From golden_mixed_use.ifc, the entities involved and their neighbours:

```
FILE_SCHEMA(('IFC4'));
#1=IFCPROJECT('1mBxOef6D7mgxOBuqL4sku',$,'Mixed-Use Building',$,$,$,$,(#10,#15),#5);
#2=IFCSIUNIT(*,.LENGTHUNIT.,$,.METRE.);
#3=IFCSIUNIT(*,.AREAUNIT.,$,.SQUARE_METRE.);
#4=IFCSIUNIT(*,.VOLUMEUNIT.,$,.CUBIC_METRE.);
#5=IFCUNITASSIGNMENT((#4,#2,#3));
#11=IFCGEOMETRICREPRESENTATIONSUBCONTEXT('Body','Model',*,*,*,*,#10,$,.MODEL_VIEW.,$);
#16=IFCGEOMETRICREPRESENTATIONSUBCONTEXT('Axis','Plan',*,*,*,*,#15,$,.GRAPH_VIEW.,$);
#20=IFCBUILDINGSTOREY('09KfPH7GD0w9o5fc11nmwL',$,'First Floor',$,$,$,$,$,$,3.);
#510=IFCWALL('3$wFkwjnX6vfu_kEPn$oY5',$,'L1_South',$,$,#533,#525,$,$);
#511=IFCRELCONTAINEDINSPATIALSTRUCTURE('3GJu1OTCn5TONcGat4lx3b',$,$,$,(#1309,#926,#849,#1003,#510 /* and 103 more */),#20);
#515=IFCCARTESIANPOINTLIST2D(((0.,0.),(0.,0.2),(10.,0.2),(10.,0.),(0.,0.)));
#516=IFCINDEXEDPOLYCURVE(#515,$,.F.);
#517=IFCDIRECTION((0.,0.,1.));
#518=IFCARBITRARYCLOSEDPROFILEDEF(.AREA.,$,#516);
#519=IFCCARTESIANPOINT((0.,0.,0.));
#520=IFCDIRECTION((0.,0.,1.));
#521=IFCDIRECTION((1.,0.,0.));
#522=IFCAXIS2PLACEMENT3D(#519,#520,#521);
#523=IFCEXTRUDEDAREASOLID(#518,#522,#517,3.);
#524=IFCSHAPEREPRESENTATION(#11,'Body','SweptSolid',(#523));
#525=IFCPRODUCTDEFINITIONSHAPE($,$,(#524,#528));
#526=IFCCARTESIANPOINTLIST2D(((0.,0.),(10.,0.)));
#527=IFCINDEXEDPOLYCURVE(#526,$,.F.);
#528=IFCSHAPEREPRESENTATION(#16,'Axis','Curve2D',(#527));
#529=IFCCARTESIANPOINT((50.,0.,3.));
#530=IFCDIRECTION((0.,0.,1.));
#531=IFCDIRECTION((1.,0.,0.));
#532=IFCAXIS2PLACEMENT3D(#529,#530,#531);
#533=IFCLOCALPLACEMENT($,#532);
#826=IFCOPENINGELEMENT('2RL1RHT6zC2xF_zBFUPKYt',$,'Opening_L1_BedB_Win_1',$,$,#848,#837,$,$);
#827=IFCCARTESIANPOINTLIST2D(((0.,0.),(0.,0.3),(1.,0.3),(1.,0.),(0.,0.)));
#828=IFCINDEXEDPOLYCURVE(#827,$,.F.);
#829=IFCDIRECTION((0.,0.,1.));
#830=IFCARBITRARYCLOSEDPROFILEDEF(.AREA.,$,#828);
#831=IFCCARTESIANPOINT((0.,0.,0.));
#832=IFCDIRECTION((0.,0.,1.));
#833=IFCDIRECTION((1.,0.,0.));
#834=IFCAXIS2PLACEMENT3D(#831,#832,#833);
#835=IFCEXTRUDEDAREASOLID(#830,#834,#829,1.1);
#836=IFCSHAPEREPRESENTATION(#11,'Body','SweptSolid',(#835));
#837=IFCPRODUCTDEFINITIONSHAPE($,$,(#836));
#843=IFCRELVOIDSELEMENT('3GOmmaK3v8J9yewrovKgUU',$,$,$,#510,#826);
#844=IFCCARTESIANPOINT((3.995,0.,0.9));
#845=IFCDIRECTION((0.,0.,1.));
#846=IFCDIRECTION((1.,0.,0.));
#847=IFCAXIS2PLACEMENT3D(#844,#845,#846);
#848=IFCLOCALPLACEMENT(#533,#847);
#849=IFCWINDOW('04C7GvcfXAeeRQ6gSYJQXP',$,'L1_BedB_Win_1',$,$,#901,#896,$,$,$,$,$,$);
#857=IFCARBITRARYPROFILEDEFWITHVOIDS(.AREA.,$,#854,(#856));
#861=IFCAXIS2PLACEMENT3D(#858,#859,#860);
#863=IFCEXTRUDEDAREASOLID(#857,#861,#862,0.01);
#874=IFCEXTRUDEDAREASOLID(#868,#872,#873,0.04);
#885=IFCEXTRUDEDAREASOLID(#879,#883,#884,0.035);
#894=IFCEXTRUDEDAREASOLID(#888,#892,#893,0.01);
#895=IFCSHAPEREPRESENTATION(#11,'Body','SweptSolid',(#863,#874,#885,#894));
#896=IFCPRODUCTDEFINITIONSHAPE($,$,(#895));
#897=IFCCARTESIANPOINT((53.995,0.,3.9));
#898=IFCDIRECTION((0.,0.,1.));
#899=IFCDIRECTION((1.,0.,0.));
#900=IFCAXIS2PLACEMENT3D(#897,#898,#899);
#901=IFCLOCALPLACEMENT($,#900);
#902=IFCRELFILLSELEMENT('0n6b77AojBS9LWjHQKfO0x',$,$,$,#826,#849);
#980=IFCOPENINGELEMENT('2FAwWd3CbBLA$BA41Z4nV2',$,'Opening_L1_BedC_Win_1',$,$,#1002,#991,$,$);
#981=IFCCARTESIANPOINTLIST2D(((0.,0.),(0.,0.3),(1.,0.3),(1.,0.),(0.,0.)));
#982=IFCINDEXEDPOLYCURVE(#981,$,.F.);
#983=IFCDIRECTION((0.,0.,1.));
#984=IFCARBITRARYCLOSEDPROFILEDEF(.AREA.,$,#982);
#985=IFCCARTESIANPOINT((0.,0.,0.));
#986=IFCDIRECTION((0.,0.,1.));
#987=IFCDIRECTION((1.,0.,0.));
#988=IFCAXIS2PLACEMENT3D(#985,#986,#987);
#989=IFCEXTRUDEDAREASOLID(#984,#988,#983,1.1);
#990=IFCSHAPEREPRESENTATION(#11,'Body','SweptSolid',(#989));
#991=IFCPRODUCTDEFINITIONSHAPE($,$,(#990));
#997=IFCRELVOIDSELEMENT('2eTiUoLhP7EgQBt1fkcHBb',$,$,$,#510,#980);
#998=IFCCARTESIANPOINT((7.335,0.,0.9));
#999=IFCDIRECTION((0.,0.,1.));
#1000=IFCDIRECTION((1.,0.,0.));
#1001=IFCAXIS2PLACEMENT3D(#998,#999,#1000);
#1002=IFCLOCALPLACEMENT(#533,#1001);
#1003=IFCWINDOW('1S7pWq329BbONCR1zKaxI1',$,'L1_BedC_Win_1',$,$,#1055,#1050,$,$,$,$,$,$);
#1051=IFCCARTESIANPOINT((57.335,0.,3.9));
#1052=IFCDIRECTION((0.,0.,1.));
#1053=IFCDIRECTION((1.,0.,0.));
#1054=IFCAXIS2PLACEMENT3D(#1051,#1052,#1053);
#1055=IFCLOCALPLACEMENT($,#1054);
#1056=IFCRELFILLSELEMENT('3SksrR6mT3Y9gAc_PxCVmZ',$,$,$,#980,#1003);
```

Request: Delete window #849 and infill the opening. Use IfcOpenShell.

```python
import ifcopenshell
import ifcopenshell.api.feature
import ifcopenshell.api.root
import ifcopenshell.geom
import ifcopenshell.util.shape

model = ifcopenshell.open("golden_mixed_use.ifc")
settings = ifcopenshell.geom.settings()


def volume(element):
    """Net volume in cubic metres, openings subtracted."""
    shape = ifcopenshell.geom.create_shape(settings, element)
    return ifcopenshell.util.shape.get_volume(shape.geometry)


window = model.by_id(849)
opening = window.FillsVoids[0].RelatingOpeningElement
wall = opening.VoidsElements[0].RelatingBuildingElement
before = volume(wall)

ifcopenshell.api.root.remove_product(model, product=window)
ifcopenshell.api.feature.remove_feature(model, feature=opening)

after = volume(wall)

print(f"wall volume {before:.3f} -> {after:.3f} m3")

model.write("golden_mixed_use_v2.ifc")
```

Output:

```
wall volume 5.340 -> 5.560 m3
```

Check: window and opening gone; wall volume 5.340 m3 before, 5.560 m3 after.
